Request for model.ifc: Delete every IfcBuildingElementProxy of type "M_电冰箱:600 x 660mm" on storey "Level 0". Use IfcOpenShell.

First a look at what the model holds.

```python
import ifcopenshell
import ifcopenshell.util.element

model = ifcopenshell.open("model.ifc")
print(model.schema)
storey = next(s for s in model.by_type("IfcBuildingStorey") if s.Name == "Level 0")
proxies = [e for e in ifcopenshell.util.element.get_decomposition(storey) if e.is_a("IfcBuildingElementProxy")]
seen = {}
for e in proxies:
    element_type = ifcopenshell.util.element.get_type(e)
    name = element_type.Name if element_type not in (None, e) else None
    seen[name] = seen.get(name, 0) + 1
for name, count in sorted(seen.items(), key=str):
    print(count, "x", name)
```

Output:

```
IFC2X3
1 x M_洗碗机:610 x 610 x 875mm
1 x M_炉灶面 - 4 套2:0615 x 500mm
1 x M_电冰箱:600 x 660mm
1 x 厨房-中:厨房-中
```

```python
import ifcopenshell
import ifcopenshell.api.root
import ifcopenshell.util.element

model = ifcopenshell.open("model.ifc")

storey = next(s for s in model.by_type("IfcBuildingStorey") if s.Name == "Level 0")
proxies = [e for e in ifcopenshell.util.element.get_decomposition(storey) if e.is_a("IfcBuildingElementProxy")]
targets = [e for e in proxies if (t := ifcopenshell.util.element.get_type(e)) not in (None, e) and t.Name == "M_电冰箱:600 x 660mm"]

for e in targets:
    ifcopenshell.api.root.remove_product(model, product=e)
print(len(targets), "removed")

model.write("model_rev.ifc")
```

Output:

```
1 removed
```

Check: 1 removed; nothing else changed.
